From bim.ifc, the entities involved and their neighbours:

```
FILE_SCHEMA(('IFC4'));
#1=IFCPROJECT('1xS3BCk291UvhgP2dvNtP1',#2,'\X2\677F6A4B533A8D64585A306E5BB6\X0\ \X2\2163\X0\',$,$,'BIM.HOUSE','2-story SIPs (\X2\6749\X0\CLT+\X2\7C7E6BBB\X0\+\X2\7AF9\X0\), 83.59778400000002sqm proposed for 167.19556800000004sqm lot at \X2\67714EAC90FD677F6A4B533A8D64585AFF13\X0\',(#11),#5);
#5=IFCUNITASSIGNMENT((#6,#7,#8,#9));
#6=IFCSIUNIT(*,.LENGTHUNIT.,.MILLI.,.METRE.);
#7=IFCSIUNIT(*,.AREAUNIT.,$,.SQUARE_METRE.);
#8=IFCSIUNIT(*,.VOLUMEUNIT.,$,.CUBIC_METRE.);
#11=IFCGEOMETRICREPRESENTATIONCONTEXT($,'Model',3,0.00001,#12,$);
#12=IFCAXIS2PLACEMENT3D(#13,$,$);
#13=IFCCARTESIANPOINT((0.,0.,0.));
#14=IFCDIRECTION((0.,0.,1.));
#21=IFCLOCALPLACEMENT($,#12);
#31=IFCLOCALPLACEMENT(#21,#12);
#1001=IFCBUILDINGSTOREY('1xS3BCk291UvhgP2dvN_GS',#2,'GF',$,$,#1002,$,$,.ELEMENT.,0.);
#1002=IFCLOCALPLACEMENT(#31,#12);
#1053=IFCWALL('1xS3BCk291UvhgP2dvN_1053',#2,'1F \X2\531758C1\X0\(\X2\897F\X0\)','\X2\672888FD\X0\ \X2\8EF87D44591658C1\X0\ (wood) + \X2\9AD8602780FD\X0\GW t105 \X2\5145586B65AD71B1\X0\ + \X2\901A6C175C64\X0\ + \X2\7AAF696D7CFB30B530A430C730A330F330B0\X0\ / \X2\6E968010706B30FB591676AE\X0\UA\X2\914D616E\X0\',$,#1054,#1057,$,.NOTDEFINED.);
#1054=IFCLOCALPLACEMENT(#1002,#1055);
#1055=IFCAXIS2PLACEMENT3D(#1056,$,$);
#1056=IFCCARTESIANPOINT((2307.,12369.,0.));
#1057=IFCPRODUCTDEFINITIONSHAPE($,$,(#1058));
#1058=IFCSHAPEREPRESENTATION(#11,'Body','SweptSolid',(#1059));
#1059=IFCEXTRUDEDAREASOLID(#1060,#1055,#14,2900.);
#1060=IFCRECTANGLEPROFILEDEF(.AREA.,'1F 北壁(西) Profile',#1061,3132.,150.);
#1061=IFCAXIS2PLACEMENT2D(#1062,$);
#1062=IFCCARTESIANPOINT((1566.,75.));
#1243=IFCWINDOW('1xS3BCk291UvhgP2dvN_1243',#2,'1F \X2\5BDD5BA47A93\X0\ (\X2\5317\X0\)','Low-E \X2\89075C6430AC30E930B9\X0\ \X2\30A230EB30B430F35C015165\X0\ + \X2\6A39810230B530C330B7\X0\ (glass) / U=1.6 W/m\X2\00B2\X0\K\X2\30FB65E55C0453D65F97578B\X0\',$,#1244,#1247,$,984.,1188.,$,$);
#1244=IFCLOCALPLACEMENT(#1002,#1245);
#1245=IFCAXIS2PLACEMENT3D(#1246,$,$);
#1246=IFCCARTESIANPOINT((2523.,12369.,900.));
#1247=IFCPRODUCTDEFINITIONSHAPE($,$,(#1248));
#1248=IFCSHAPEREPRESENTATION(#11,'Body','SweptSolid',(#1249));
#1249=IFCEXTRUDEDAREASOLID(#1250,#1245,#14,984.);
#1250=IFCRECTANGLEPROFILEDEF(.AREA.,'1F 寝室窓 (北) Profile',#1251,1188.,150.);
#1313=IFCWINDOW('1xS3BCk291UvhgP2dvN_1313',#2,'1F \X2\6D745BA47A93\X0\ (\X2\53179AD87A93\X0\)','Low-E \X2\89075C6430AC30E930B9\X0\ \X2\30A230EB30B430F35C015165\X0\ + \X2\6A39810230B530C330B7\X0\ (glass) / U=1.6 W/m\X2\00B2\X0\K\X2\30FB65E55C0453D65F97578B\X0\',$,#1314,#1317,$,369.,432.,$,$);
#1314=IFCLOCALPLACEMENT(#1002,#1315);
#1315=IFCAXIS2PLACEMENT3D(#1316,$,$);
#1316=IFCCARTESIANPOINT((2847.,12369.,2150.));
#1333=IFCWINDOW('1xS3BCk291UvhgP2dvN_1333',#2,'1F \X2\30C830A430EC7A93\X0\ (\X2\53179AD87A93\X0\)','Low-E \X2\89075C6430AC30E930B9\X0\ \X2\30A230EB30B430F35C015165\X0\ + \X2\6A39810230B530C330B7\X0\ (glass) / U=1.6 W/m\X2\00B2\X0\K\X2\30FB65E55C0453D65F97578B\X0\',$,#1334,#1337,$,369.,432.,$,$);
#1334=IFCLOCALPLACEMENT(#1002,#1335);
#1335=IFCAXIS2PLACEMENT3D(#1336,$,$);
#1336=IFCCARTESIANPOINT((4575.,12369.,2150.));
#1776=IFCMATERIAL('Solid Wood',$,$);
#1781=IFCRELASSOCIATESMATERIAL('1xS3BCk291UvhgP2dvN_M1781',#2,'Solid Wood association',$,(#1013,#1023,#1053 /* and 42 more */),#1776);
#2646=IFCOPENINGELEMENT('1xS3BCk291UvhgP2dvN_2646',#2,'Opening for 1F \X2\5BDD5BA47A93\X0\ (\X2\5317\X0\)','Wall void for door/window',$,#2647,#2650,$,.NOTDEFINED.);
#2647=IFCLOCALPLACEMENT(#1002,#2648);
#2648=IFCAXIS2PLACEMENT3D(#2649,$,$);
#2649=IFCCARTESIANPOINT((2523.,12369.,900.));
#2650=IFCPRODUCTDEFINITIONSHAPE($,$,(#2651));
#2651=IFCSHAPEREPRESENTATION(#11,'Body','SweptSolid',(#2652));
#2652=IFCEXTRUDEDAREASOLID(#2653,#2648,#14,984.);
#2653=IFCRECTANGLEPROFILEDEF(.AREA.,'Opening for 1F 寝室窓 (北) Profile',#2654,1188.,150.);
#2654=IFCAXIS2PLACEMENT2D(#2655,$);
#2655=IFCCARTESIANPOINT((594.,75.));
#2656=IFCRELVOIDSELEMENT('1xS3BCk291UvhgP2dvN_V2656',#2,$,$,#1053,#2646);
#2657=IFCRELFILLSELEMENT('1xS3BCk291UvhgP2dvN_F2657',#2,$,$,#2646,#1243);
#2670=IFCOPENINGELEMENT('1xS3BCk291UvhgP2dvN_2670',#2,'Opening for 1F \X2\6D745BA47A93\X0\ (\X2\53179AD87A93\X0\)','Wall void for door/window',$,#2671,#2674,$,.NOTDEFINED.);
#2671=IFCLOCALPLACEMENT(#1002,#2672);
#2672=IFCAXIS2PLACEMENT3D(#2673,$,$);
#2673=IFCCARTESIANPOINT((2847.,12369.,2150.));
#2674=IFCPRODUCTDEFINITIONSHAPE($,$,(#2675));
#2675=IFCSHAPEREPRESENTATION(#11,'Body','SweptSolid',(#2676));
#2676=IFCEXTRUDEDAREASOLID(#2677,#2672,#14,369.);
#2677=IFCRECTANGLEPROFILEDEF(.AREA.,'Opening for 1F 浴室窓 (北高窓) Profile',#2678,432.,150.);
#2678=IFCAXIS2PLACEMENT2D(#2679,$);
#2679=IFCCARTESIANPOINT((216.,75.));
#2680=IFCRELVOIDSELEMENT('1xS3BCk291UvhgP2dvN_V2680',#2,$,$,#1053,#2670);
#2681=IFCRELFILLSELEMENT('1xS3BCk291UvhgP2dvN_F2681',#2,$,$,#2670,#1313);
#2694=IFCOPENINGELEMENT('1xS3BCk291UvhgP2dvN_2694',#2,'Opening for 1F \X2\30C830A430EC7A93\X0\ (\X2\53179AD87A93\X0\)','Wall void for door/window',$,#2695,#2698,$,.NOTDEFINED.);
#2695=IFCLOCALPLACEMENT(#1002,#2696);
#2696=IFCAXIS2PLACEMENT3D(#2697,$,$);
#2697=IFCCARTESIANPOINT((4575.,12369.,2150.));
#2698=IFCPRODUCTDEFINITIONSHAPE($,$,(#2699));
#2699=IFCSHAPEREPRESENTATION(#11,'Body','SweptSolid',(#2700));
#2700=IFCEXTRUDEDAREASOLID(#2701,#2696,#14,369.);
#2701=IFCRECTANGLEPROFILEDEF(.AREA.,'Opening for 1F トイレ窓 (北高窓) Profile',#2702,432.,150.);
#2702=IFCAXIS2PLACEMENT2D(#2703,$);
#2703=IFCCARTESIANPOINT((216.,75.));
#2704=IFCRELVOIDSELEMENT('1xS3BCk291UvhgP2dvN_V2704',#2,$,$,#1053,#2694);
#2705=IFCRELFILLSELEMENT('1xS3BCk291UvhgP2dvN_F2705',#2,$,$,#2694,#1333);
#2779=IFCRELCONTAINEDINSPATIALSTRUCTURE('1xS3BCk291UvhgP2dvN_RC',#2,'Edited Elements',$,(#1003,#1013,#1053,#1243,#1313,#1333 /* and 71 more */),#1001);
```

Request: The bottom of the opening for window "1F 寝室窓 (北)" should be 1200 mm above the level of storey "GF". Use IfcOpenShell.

```python
import numpy as np
import ifcopenshell
import ifcopenshell.api.geometry
import ifcopenshell.geom
import ifcopenshell.util.element
import ifcopenshell.util.placement
import ifcopenshell.util.shape
import ifcopenshell.util.unit

model = ifcopenshell.open("bim.ifc")
unit_scale = ifcopenshell.util.unit.calculate_unit_scale(model)

window = model.by_guid("1xS3BCk291UvhgP2dvN_1243")
opening = window.FillsVoids[0].RelatingOpeningElement
storey = ifcopenshell.util.element.get_container(window, ifc_class="IfcBuildingStorey")
level = ifcopenshell.util.placement.get_local_placement(storey.ObjectPlacement)[2, 3]

# The opening's origin need not be at the sill, so measure its lowest point.
shape = ifcopenshell.geom.create_shape(ifcopenshell.geom.settings(), opening)
bottom = ifcopenshell.util.shape.get_shape_bottom_elevation(shape, shape.geometry) / unit_scale
dz = level + 1.2 / unit_scale - bottom

shift = np.array([0.0, 0.0, dz])
# The window is not placed relative to its opening, so move both.
for product in (opening, window):
    matrix = ifcopenshell.util.placement.get_local_placement(product.ObjectPlacement)
    matrix[:3, 3] += shift
    ifcopenshell.api.geometry.edit_object_placement(model, product=product, matrix=matrix, is_si=False)

print(f"moved by {dz * unit_scale:+.3f} m")

model.write("bim_edited.ifc")
```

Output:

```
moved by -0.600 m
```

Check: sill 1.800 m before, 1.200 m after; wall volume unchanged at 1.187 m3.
